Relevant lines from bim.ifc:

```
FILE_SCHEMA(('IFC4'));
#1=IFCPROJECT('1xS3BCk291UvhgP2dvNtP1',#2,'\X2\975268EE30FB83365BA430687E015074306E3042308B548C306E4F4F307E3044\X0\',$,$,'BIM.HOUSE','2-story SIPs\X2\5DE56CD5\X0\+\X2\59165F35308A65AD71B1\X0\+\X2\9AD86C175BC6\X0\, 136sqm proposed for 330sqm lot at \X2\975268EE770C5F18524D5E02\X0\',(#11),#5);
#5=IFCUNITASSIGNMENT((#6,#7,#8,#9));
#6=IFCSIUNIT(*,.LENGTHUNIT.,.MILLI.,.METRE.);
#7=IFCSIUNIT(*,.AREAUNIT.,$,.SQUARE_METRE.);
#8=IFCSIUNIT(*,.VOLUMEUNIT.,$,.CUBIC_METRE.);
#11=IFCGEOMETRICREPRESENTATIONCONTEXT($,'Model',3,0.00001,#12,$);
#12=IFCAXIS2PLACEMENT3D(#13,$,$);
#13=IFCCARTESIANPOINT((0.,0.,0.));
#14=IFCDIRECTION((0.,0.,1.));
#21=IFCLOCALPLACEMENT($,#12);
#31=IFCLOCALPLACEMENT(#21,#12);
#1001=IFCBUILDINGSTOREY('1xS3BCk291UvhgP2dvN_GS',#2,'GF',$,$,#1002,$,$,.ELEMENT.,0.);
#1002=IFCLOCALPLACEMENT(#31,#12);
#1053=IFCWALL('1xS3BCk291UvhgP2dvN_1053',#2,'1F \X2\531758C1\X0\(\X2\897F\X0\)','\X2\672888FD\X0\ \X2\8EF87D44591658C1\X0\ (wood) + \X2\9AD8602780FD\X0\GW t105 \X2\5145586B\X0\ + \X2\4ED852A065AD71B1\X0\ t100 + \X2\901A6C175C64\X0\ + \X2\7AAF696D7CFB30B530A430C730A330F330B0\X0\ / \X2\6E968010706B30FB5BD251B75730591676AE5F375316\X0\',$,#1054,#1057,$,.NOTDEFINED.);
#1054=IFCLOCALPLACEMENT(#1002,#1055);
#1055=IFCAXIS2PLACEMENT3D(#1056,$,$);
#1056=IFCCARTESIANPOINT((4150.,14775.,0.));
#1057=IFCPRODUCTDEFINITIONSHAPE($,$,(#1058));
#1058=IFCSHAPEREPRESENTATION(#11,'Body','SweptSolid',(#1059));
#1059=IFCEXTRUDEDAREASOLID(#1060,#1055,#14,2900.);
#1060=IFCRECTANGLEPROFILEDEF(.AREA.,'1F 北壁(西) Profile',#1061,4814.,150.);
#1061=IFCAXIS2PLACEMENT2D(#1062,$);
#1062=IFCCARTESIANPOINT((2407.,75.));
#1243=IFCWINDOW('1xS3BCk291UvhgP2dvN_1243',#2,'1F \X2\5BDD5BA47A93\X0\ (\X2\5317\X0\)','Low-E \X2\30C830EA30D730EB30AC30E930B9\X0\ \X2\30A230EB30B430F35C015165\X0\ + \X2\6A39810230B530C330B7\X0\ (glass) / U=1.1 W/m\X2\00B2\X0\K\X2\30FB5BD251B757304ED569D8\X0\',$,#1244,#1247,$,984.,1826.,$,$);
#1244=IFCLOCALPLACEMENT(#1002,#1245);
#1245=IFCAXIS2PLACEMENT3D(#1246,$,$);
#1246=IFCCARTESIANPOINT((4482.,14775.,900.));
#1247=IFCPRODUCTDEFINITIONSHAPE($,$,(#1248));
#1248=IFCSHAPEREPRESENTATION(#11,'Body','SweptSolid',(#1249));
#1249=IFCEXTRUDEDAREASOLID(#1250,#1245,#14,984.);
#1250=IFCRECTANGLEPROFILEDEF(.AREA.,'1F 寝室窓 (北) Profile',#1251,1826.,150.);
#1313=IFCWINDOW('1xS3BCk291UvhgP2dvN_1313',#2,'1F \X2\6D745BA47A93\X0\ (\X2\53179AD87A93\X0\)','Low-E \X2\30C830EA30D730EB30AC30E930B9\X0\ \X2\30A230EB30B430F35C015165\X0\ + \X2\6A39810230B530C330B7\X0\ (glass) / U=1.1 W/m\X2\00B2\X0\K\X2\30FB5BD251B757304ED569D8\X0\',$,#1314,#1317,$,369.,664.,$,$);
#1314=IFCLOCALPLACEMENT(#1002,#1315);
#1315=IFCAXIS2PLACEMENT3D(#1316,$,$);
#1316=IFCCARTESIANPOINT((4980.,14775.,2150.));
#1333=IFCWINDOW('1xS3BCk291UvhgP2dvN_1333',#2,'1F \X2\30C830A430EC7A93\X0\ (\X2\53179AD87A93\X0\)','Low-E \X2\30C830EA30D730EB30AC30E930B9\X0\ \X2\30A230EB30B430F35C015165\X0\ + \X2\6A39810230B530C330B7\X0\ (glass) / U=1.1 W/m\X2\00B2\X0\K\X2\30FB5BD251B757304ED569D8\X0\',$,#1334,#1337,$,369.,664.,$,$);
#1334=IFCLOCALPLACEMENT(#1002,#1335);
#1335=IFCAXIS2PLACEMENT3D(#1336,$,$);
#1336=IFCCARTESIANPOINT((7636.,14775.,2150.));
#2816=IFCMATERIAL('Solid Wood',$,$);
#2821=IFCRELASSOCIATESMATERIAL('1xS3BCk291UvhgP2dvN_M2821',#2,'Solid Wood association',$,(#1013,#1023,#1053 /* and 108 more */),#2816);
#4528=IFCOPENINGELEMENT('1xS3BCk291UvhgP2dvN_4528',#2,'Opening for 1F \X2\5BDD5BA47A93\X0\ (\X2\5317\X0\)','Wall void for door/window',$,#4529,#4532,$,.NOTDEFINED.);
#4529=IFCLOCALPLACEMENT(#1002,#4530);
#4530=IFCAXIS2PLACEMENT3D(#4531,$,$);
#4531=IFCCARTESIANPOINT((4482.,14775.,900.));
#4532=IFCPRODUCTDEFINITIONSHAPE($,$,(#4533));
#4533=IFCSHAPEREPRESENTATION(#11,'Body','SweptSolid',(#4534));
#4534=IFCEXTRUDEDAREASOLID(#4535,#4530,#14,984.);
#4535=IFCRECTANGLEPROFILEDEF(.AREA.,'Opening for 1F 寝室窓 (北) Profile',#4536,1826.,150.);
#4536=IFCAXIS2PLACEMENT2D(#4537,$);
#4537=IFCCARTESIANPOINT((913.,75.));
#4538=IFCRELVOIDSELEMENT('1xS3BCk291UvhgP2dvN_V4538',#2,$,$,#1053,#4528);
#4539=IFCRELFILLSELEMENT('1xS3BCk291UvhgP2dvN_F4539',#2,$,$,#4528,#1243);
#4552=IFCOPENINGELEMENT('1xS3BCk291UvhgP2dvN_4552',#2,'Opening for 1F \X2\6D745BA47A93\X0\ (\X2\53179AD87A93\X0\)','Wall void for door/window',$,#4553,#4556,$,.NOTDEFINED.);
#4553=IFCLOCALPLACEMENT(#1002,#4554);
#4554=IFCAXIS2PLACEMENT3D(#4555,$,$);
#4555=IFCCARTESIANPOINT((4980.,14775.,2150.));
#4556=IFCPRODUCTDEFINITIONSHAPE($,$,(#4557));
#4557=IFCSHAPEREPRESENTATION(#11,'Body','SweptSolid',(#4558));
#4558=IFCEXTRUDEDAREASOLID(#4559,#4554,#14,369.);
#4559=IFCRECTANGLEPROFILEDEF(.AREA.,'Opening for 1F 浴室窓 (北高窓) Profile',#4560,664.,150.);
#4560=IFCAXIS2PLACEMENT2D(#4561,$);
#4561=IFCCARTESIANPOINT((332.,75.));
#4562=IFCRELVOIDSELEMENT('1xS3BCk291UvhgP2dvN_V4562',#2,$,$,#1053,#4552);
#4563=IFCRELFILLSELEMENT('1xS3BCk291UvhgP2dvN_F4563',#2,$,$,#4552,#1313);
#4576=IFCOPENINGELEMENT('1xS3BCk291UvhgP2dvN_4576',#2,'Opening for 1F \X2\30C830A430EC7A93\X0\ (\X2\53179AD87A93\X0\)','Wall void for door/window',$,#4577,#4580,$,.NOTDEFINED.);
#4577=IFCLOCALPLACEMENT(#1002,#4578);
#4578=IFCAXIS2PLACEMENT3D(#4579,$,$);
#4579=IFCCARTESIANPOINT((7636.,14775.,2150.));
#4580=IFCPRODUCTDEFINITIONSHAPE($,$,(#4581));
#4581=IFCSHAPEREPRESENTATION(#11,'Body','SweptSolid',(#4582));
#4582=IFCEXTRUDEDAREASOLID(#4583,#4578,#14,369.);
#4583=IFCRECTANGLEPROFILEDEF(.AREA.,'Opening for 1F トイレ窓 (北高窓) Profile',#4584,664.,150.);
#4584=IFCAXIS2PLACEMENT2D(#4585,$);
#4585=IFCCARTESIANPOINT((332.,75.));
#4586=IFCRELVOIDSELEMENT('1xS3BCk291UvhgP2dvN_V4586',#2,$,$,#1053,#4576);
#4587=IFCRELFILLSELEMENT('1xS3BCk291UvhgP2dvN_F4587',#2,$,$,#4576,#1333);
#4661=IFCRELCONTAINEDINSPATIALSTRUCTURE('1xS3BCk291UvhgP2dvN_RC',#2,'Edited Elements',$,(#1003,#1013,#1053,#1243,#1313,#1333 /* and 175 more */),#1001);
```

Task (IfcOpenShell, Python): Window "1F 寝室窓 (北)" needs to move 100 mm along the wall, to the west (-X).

```python
import ifcopenshell
import ifcopenshell.api.geometry
import ifcopenshell.util.placement
import ifcopenshell.util.unit

model = ifcopenshell.open("bim.ifc")
unit_scale = ifcopenshell.util.unit.calculate_unit_scale(model)

window = model.by_guid("1xS3BCk291UvhgP2dvN_1243")
opening = window.FillsVoids[0].RelatingOpeningElement
wall = opening.VoidsElements[0].RelatingBuildingElement

wall_matrix = ifcopenshell.util.placement.get_local_placement(wall.ObjectPlacement)
shift = wall_matrix[:3, 0] * -0.1 / unit_scale
before = ifcopenshell.util.placement.get_local_placement(window.ObjectPlacement)[:3, 3].copy()

# The window is not placed relative to its opening, so move both.
for product in (opening, window):
    matrix = ifcopenshell.util.placement.get_local_placement(product.ObjectPlacement)
    matrix[:3, 3] += shift
    ifcopenshell.api.geometry.edit_object_placement(model, product=product, matrix=matrix, is_si=False)

after = ifcopenshell.util.placement.get_local_placement(window.ObjectPlacement)[:3, 3]
print("window moved by", (after - before).round(3) + 0.0)

model.write("bim_updated.ifc")
```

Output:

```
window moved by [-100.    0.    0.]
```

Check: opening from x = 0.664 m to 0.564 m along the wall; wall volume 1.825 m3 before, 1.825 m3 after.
